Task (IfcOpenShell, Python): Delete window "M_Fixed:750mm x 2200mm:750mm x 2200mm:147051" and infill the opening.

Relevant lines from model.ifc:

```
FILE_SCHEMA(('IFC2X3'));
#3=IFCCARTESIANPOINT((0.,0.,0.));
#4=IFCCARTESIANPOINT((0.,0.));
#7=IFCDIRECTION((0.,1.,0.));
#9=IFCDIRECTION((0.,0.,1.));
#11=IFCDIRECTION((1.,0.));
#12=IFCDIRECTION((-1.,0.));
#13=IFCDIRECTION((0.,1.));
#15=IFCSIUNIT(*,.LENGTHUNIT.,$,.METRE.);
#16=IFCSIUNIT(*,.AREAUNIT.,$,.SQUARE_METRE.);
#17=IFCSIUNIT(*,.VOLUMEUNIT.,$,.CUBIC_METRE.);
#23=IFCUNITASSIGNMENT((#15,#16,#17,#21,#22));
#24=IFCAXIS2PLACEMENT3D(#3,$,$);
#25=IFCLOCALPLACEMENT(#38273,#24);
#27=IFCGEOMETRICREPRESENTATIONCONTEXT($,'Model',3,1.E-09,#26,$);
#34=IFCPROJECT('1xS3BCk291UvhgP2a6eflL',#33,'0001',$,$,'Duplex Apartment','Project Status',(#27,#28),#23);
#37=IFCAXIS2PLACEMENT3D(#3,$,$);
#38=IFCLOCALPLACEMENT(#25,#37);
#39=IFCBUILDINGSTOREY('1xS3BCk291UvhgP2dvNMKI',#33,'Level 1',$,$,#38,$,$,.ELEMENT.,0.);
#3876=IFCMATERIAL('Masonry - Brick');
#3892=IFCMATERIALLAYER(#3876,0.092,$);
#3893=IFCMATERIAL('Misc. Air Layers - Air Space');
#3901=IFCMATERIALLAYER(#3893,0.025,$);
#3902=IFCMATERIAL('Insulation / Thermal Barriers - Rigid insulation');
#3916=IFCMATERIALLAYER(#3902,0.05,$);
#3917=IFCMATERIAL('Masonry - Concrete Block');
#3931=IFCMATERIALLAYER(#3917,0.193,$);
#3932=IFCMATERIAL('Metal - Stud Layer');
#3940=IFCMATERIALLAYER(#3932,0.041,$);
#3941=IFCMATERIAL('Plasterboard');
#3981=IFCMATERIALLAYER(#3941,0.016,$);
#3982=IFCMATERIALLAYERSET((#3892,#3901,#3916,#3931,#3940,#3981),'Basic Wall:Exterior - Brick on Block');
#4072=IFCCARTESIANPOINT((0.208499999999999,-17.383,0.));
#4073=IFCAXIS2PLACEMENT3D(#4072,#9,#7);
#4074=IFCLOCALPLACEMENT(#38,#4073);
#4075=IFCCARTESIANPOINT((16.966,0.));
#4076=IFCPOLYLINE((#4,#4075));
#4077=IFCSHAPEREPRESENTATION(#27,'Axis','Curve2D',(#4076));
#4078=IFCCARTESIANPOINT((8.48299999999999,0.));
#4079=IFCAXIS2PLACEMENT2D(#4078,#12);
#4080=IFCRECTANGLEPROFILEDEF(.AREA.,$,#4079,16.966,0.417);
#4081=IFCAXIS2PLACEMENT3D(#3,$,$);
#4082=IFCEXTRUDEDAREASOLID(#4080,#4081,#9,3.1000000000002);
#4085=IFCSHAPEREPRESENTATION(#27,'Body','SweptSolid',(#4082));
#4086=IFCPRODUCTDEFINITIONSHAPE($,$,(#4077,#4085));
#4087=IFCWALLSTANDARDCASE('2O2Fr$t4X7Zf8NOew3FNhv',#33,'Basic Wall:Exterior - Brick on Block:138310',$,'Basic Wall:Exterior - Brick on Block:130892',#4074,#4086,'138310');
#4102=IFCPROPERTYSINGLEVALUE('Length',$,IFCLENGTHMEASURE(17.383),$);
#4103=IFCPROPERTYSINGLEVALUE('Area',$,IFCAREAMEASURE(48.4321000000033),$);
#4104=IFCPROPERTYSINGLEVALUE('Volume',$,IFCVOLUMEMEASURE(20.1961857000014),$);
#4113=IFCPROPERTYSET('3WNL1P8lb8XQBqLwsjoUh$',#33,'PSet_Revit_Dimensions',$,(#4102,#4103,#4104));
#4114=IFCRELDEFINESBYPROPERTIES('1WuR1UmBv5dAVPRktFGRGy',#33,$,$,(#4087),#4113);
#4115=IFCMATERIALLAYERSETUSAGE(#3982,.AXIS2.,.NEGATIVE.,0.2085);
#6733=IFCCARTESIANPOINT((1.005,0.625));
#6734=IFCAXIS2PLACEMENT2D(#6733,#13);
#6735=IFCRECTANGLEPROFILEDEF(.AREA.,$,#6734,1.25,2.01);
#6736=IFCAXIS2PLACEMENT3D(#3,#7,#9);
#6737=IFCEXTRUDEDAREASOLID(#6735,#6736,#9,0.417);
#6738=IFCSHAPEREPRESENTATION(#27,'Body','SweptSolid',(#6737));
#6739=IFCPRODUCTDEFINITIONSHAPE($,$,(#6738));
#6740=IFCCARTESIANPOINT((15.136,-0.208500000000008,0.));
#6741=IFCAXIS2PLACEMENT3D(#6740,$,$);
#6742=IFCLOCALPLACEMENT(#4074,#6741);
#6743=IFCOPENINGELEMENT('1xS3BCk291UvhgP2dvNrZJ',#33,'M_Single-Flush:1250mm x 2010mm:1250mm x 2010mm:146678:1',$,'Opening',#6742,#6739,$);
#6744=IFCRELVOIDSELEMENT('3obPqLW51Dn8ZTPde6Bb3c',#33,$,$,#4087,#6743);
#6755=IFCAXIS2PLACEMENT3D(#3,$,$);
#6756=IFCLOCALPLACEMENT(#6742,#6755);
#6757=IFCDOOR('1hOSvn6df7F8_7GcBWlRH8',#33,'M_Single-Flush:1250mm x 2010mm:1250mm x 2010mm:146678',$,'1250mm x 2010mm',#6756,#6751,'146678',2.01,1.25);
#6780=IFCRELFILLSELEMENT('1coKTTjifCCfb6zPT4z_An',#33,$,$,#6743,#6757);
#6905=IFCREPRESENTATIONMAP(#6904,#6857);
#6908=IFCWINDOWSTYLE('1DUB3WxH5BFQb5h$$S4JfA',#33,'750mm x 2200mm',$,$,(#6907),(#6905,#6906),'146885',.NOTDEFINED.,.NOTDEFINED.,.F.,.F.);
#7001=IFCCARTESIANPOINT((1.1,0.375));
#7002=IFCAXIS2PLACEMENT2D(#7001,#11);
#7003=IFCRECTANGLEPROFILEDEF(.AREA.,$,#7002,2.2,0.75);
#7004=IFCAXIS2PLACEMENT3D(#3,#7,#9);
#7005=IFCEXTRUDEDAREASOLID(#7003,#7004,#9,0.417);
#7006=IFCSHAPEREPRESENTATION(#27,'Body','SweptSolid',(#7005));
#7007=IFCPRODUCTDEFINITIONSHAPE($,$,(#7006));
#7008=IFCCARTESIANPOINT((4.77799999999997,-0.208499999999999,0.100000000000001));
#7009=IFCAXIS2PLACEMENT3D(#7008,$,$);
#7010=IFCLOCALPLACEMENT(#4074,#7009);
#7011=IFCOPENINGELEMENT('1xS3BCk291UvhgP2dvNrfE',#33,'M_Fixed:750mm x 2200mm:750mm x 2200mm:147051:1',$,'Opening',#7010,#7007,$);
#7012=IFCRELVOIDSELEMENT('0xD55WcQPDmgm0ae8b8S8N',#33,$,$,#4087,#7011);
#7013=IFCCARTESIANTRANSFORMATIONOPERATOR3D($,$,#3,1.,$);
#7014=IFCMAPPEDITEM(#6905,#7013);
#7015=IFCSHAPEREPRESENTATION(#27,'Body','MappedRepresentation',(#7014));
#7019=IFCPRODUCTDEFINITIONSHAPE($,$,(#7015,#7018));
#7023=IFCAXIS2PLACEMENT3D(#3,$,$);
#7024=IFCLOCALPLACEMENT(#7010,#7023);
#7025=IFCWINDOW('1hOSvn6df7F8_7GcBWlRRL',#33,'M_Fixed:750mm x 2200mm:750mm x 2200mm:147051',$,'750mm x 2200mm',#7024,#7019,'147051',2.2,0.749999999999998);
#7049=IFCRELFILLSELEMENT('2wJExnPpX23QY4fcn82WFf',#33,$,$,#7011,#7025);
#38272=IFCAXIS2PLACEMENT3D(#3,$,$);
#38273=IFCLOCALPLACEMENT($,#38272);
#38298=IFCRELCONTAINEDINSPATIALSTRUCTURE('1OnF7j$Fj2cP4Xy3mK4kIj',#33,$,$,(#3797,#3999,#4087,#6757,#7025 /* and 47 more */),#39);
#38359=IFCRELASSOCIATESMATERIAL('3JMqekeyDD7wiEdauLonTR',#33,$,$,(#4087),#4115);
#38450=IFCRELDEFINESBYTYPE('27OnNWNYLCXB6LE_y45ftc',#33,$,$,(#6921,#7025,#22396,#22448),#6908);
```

```python
import ifcopenshell
import ifcopenshell.api.feature
import ifcopenshell.api.pset
import ifcopenshell.api.root
import ifcopenshell.geom
import ifcopenshell.util.element
import ifcopenshell.util.shape
import ifcopenshell.util.unit

model = ifcopenshell.open("model.ifc")
area_scale = ifcopenshell.util.unit.calculate_unit_scale(model, "AREAUNIT")
volume_scale = ifcopenshell.util.unit.calculate_unit_scale(model, "VOLUMEUNIT")
settings = ifcopenshell.geom.settings()


def volume(element):
    """Net volume in cubic metres, openings subtracted."""
    shape = ifcopenshell.geom.create_shape(settings, element)
    return ifcopenshell.util.shape.get_volume(shape.geometry)


window = model.by_guid("1hOSvn6df7F8_7GcBWlRRL")
opening = window.FillsVoids[0].RelatingOpeningElement
wall = opening.VoidsElements[0].RelatingBuildingElement
before = volume(wall)

ifcopenshell.api.root.remove_product(model, product=window)
ifcopenshell.api.feature.remove_feature(model, feature=opening)

after = volume(wall)
thickness = 0.417  # wall thickness in metres

# Update the wall's stored quantities.
pset = model.by_id(ifcopenshell.util.element.get_pset(wall, "PSet_Revit_Dimensions", should_inherit=False)["id"])
ifcopenshell.api.pset.edit_pset(model, pset=pset, properties={
    "Area": model.create_entity("IfcAreaMeasure", after / thickness / area_scale),
    "Volume": model.create_entity("IfcVolumeMeasure", after / volume_scale),
})

print(f"wall volume {before:.3f} -> {after:.3f} m3")

model.write("model-out.ifc")
```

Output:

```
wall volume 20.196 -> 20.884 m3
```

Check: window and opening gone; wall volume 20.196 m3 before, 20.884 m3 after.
